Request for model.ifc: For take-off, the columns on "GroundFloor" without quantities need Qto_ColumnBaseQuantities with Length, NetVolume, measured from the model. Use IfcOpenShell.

First a look at what the model holds.

```python
import ifcopenshell
import ifcopenshell.util.element
import ifcopenshell.util.unit

model = ifcopenshell.open("model.ifc")
print(model.schema)
for unit_type in ("LENGTHUNIT", "AREAUNIT", "VOLUMEUNIT"):
    print(unit_type, ifcopenshell.util.unit.calculate_unit_scale(model, unit_type))
storey = next(s for s in model.by_type("IfcBuildingStorey") if s.Name == "GroundFloor")
columns = [e for e in ifcopenshell.util.element.get_decomposition(storey) if e.is_a("IfcColumn")]
for e in sorted(columns, key=lambda e: e.id()):
    print(e.id(), e.is_a(), e.Name, list(ifcopenshell.util.element.get_psets(e, qtos_only=True)), sep=" | ")
```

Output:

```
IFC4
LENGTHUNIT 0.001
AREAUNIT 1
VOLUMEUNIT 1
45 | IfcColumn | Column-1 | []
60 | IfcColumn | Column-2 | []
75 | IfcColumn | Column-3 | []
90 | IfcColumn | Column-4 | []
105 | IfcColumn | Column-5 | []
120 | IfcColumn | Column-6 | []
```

```python
import ifcopenshell
import ifcopenshell.api.pset
import ifcopenshell.geom
import ifcopenshell.util.element
import ifcopenshell.util.shape
import ifcopenshell.util.unit

model = ifcopenshell.open("model.ifc")
unit_scale = ifcopenshell.util.unit.calculate_unit_scale(model)
volume_scale = ifcopenshell.util.unit.calculate_unit_scale(model, "VOLUMEUNIT")
settings = ifcopenshell.geom.settings()

storey = next(s for s in model.by_type("IfcBuildingStorey") if s.Name == "GroundFloor")
columns = [e for e in ifcopenshell.util.element.get_decomposition(storey) if e.is_a("IfcColumn")]

for e in sorted(columns, key=lambda e: e.id()):
    if ifcopenshell.util.element.get_psets(e, qtos_only=True, should_inherit=False):
        continue
    # Geometry comes back in metres, in the element's own axes.
    shape = ifcopenshell.geom.create_shape(settings, e)
    values = {
        "Length": ifcopenshell.util.shape.get_z(shape.geometry) / unit_scale,
        "NetVolume": ifcopenshell.util.shape.get_volume(shape.geometry) / volume_scale,
    }
    qto = ifcopenshell.api.pset.add_qto(model, product=e, name="Qto_ColumnBaseQuantities")
    ifcopenshell.api.pset.edit_qto(model, qto=qto, properties=values)
    print(e.id(), {k: round(v, 3) for k, v in values.items()})

model.write("model_rev.ifc")
```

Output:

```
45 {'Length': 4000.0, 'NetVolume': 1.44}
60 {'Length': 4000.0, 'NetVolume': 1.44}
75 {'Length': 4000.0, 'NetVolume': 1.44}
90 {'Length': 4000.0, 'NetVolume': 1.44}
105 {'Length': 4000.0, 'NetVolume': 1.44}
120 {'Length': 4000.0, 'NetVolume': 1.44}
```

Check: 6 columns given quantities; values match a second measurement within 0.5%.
